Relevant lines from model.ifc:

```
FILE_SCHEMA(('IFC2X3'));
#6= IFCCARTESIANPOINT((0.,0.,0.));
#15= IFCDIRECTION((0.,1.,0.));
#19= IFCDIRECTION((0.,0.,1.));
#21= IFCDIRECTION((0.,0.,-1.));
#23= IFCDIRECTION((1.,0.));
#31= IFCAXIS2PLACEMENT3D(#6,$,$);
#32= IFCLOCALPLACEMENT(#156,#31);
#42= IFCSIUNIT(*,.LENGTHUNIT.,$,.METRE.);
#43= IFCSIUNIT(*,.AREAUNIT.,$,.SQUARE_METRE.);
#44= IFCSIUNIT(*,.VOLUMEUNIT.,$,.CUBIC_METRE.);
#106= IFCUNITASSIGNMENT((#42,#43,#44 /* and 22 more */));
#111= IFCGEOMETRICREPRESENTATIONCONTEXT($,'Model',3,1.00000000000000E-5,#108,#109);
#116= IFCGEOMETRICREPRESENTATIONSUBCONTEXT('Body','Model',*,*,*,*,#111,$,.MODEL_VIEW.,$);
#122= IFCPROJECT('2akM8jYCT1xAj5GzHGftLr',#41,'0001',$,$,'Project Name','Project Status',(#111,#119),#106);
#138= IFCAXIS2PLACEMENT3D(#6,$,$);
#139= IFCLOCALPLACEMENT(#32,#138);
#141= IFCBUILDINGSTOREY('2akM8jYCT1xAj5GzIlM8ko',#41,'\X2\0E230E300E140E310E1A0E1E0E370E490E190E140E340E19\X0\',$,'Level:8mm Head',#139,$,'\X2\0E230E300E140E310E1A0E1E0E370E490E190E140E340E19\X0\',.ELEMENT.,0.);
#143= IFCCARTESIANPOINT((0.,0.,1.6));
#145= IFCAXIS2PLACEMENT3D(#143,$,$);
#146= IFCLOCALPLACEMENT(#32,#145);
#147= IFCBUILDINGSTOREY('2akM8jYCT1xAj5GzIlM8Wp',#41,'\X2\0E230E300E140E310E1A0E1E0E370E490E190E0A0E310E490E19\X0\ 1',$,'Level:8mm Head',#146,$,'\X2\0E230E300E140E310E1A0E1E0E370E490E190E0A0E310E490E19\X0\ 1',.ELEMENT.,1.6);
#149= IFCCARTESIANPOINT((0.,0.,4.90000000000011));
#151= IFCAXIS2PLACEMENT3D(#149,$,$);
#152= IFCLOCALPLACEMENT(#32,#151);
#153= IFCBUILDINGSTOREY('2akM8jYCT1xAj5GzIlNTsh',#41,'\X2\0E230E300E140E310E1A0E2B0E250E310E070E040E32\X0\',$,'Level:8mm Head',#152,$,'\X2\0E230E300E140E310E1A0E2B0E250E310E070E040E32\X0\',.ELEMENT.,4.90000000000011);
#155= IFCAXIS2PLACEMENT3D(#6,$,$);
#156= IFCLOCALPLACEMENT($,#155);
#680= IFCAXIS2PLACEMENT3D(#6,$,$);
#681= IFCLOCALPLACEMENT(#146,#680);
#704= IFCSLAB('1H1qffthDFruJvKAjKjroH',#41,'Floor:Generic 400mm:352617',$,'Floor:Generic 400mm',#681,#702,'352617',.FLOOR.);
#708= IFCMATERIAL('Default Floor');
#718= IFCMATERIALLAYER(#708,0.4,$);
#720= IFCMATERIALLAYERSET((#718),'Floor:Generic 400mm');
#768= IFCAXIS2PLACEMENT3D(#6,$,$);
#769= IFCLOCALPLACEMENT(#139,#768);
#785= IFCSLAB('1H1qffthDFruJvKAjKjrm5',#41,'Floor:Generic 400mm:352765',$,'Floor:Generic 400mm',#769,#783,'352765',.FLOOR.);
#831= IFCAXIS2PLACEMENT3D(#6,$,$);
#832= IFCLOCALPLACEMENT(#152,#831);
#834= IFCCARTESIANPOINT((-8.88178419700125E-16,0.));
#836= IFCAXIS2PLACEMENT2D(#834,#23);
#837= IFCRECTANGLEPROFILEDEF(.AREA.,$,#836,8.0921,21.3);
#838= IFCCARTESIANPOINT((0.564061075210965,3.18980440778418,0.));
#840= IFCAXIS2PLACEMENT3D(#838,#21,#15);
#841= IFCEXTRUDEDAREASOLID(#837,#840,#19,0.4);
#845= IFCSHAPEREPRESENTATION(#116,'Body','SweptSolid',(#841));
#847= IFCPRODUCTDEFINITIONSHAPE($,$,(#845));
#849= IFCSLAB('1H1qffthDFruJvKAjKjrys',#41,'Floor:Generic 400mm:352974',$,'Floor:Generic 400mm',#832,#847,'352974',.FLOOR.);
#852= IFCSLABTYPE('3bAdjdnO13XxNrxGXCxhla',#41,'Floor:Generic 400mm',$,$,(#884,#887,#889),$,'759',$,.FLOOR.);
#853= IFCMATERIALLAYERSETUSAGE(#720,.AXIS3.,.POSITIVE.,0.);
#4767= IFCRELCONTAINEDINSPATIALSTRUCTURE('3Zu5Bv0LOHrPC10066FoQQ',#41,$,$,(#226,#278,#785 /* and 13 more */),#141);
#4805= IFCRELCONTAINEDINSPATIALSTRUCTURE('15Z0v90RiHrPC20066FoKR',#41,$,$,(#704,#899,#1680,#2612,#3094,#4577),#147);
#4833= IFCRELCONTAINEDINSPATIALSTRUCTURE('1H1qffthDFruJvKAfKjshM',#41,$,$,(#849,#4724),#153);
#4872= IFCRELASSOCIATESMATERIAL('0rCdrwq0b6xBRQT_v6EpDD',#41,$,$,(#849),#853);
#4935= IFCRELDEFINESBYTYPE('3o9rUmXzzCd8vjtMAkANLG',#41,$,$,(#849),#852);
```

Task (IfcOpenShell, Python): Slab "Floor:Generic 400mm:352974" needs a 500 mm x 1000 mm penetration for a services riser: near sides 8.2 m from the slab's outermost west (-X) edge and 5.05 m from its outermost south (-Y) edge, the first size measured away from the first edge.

```python
import numpy as np
import ifcopenshell
import ifcopenshell.api.feature
import ifcopenshell.api.geometry
import ifcopenshell.api.root
import ifcopenshell.geom
import ifcopenshell.util.placement
import ifcopenshell.util.representation
import ifcopenshell.util.shape
import ifcopenshell.util.unit

model = ifcopenshell.open("model.ifc")
unit_scale = ifcopenshell.util.unit.calculate_unit_scale(model)
settings = ifcopenshell.geom.settings()


def volume(element):
    """Net volume in cubic metres, openings subtracted."""
    shape = ifcopenshell.geom.create_shape(settings, element)
    return ifcopenshell.util.shape.get_volume(shape.geometry)


slab = model.by_id(849)
before = volume(slab)

# Extent in the slab's own axes, in metres. The edges named are its -X and -Y sides.
slab_shape = ifcopenshell.geom.create_shape(settings, slab)
vertices = ifcopenshell.util.shape.get_vertices(slab_shape.geometry)
x_min, y_min, bottom = vertices.min(axis=0)
top = vertices[:, 2].max()

opening = ifcopenshell.api.root.create_entity(model, ifc_class="IfcOpeningElement", name="Services riser opening")
context = ifcopenshell.util.representation.get_context(model, "Model", "Body", "MODEL_VIEW")
width, depth = 0.5, 1
outline = [(0.0, 0.0), (width, 0.0), (width, depth), (0.0, depth), (0.0, 0.0)]
# Overshoot both faces by 50 mm so the cut is clean.
shape = ifcopenshell.api.geometry.add_slab_representation(
    model, context=context, depth=top - bottom + 0.1, polyline=outline
)
ifcopenshell.api.geometry.assign_representation(model, product=opening, representation=shape)

matrix = ifcopenshell.util.placement.get_local_placement(slab.ObjectPlacement)
matrix[:, 3] = matrix @ np.append(np.array([x_min + 8.2, y_min + 5.05, bottom - 0.05]) / unit_scale, 1.0)
ifcopenshell.api.geometry.edit_object_placement(model, product=opening, matrix=matrix, is_si=False)
ifcopenshell.api.feature.add_feature(model, feature=opening, element=slab)

after = volume(slab)

print(f"slab volume {before:.3f} -> {after:.3f} m3")

model.write("model_rev.ifc")
```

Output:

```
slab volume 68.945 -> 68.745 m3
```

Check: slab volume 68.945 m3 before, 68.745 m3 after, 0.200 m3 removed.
